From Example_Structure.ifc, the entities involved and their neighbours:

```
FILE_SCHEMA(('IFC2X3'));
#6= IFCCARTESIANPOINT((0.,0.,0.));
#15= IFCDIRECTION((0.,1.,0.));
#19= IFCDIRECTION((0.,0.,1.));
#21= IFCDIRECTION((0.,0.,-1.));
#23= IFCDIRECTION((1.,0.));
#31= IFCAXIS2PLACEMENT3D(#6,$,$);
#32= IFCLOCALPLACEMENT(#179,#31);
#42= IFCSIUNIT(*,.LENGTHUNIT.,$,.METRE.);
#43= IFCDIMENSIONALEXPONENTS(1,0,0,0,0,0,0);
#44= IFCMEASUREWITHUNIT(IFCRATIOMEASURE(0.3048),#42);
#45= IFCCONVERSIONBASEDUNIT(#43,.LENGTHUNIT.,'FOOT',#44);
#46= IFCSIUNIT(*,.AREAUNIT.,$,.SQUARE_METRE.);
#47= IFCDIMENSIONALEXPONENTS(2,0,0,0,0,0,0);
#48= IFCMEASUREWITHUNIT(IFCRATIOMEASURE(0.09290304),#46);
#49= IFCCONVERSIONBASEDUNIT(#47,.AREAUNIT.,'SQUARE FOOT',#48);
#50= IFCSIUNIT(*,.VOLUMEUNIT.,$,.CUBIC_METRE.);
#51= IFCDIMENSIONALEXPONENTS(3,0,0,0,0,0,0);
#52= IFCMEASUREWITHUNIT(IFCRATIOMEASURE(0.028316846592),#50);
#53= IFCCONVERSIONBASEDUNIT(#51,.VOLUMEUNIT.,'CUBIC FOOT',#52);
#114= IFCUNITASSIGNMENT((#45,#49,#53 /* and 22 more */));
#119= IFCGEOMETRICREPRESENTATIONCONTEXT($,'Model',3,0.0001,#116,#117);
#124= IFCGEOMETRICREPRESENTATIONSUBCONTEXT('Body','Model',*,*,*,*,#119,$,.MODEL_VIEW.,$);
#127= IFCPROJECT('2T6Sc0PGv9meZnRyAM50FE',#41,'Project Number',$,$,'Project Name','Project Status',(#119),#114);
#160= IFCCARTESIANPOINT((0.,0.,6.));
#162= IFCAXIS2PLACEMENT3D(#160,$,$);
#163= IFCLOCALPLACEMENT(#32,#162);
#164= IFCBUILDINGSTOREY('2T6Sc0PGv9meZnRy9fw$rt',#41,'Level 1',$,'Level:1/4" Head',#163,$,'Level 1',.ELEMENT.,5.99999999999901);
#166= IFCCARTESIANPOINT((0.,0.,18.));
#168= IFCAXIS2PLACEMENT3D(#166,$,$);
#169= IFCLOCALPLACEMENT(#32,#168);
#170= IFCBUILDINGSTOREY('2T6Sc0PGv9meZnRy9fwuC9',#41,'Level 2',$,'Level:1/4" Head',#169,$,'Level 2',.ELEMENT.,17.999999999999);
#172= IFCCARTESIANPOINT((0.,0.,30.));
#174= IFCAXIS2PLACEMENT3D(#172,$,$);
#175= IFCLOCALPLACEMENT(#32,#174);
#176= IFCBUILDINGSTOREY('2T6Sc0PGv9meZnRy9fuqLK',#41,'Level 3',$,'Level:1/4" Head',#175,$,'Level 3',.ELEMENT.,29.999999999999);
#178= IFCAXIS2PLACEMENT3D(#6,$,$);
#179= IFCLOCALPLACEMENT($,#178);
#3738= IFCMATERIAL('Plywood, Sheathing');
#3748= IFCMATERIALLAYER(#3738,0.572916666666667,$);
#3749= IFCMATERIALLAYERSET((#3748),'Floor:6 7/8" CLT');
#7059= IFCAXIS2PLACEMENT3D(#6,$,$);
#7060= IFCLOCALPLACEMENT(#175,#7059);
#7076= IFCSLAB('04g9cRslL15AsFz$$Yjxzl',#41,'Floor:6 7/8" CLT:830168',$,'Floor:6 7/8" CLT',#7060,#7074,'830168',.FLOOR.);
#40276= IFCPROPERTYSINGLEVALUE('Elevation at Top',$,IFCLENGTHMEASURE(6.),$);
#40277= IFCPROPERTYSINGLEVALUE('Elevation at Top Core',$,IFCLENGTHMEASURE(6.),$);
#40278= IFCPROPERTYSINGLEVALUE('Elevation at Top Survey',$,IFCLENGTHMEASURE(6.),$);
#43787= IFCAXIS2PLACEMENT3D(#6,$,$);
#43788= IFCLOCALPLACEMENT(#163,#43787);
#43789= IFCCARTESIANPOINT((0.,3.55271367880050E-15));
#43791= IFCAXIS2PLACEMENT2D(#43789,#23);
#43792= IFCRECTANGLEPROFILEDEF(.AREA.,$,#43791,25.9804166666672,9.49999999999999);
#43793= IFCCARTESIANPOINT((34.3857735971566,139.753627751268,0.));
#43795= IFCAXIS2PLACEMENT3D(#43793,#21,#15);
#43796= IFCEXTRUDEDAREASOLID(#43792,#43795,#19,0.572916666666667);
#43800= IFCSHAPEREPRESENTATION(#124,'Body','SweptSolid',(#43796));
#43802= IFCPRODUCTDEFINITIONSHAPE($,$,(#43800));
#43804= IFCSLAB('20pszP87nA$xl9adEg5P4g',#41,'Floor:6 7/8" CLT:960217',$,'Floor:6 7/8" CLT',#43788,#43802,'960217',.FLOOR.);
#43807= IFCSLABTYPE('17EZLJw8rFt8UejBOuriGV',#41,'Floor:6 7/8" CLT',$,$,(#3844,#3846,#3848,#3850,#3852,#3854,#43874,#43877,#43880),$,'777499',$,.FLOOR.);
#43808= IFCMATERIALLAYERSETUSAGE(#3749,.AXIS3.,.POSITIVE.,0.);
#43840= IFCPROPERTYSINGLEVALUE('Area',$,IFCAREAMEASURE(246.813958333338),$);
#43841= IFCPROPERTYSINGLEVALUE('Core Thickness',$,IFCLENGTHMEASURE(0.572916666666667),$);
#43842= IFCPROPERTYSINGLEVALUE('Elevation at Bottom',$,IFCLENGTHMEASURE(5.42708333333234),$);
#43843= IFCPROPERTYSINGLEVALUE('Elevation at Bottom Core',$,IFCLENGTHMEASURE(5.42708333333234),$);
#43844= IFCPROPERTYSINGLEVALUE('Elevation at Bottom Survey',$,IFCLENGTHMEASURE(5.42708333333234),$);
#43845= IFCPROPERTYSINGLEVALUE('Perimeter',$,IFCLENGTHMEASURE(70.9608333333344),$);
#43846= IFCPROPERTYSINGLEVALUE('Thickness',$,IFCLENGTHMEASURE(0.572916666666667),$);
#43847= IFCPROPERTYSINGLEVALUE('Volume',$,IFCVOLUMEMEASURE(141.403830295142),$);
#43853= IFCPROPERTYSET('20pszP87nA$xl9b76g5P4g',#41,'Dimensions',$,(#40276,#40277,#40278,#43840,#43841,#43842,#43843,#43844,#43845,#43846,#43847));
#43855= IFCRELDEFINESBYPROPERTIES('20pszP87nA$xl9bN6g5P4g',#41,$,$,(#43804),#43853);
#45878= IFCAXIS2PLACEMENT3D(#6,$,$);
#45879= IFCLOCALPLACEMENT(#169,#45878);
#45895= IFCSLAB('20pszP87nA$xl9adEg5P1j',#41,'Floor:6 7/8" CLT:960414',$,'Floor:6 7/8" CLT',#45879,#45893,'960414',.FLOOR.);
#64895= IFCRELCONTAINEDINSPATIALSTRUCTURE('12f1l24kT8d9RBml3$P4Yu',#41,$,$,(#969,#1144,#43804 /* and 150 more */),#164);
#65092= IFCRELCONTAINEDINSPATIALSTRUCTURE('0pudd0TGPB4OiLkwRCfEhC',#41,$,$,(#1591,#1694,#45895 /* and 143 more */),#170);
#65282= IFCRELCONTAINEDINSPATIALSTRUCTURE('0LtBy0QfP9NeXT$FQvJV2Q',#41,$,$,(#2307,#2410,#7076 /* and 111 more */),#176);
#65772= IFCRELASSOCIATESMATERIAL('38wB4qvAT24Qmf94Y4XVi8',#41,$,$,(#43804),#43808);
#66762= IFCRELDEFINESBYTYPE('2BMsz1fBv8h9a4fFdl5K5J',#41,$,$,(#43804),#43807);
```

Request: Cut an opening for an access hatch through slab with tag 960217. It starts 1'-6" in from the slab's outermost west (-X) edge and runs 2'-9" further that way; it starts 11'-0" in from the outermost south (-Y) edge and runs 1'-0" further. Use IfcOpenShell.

```python
import numpy as np
import ifcopenshell
import ifcopenshell.api.feature
import ifcopenshell.api.geometry
import ifcopenshell.api.pset
import ifcopenshell.api.root
import ifcopenshell.geom
import ifcopenshell.util.element
import ifcopenshell.util.placement
import ifcopenshell.util.representation
import ifcopenshell.util.shape
import ifcopenshell.util.unit

model = ifcopenshell.open("Example_Structure.ifc")
unit_scale = ifcopenshell.util.unit.calculate_unit_scale(model)
area_scale = ifcopenshell.util.unit.calculate_unit_scale(model, "AREAUNIT")
volume_scale = ifcopenshell.util.unit.calculate_unit_scale(model, "VOLUMEUNIT")
settings = ifcopenshell.geom.settings()


def volume(element):
    """Net volume in cubic metres, openings subtracted."""
    shape = ifcopenshell.geom.create_shape(settings, element)
    return ifcopenshell.util.shape.get_volume(shape.geometry)


slab = model.by_guid("20pszP87nA$xl9adEg5P4g")
before = volume(slab)

# Extent in the slab's own axes, in metres. The edges named are its -X and -Y sides.
slab_shape = ifcopenshell.geom.create_shape(settings, slab)
vertices = ifcopenshell.util.shape.get_vertices(slab_shape.geometry)
x_min, y_min, bottom = vertices.min(axis=0)
top = vertices[:, 2].max()

opening = ifcopenshell.api.root.create_entity(model, ifc_class="IfcOpeningElement", name="Access hatch opening")
context = ifcopenshell.util.representation.get_context(model, "Model", "Body", "MODEL_VIEW")
width, depth = 0.8382, 0.3048
outline = [(0.0, 0.0), (width, 0.0), (width, depth), (0.0, depth), (0.0, 0.0)]
# Overshoot both faces by 50 mm so the cut is clean.
shape = ifcopenshell.api.geometry.add_slab_representation(
    model, context=context, depth=top - bottom + 0.1, polyline=outline
)
ifcopenshell.api.geometry.assign_representation(model, product=opening, representation=shape)

matrix = ifcopenshell.util.placement.get_local_placement(slab.ObjectPlacement)
matrix[:, 3] = matrix @ np.append(np.array([x_min + 0.4572, y_min + 3.3528, bottom - 0.05]) / unit_scale, 1.0)
ifcopenshell.api.geometry.edit_object_placement(model, product=opening, matrix=matrix, is_si=False)
ifcopenshell.api.feature.add_feature(model, feature=opening, element=slab)

after = volume(slab)

# Update the slab's stored quantities.
pset = model.by_id(ifcopenshell.util.element.get_pset(slab, "Dimensions", should_inherit=False)["id"])
ifcopenshell.api.pset.edit_pset(model, pset=pset, properties={
    "Area": model.create_entity("IfcAreaMeasure", after / (top - bottom) / area_scale),
    "Volume": model.create_entity("IfcVolumeMeasure", after / volume_scale),
})

print(f"slab volume {before:.3f} -> {after:.3f} m3")

model.write("Example_Structure_v2.ifc")
```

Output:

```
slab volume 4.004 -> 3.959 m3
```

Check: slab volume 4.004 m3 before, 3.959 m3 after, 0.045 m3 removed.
